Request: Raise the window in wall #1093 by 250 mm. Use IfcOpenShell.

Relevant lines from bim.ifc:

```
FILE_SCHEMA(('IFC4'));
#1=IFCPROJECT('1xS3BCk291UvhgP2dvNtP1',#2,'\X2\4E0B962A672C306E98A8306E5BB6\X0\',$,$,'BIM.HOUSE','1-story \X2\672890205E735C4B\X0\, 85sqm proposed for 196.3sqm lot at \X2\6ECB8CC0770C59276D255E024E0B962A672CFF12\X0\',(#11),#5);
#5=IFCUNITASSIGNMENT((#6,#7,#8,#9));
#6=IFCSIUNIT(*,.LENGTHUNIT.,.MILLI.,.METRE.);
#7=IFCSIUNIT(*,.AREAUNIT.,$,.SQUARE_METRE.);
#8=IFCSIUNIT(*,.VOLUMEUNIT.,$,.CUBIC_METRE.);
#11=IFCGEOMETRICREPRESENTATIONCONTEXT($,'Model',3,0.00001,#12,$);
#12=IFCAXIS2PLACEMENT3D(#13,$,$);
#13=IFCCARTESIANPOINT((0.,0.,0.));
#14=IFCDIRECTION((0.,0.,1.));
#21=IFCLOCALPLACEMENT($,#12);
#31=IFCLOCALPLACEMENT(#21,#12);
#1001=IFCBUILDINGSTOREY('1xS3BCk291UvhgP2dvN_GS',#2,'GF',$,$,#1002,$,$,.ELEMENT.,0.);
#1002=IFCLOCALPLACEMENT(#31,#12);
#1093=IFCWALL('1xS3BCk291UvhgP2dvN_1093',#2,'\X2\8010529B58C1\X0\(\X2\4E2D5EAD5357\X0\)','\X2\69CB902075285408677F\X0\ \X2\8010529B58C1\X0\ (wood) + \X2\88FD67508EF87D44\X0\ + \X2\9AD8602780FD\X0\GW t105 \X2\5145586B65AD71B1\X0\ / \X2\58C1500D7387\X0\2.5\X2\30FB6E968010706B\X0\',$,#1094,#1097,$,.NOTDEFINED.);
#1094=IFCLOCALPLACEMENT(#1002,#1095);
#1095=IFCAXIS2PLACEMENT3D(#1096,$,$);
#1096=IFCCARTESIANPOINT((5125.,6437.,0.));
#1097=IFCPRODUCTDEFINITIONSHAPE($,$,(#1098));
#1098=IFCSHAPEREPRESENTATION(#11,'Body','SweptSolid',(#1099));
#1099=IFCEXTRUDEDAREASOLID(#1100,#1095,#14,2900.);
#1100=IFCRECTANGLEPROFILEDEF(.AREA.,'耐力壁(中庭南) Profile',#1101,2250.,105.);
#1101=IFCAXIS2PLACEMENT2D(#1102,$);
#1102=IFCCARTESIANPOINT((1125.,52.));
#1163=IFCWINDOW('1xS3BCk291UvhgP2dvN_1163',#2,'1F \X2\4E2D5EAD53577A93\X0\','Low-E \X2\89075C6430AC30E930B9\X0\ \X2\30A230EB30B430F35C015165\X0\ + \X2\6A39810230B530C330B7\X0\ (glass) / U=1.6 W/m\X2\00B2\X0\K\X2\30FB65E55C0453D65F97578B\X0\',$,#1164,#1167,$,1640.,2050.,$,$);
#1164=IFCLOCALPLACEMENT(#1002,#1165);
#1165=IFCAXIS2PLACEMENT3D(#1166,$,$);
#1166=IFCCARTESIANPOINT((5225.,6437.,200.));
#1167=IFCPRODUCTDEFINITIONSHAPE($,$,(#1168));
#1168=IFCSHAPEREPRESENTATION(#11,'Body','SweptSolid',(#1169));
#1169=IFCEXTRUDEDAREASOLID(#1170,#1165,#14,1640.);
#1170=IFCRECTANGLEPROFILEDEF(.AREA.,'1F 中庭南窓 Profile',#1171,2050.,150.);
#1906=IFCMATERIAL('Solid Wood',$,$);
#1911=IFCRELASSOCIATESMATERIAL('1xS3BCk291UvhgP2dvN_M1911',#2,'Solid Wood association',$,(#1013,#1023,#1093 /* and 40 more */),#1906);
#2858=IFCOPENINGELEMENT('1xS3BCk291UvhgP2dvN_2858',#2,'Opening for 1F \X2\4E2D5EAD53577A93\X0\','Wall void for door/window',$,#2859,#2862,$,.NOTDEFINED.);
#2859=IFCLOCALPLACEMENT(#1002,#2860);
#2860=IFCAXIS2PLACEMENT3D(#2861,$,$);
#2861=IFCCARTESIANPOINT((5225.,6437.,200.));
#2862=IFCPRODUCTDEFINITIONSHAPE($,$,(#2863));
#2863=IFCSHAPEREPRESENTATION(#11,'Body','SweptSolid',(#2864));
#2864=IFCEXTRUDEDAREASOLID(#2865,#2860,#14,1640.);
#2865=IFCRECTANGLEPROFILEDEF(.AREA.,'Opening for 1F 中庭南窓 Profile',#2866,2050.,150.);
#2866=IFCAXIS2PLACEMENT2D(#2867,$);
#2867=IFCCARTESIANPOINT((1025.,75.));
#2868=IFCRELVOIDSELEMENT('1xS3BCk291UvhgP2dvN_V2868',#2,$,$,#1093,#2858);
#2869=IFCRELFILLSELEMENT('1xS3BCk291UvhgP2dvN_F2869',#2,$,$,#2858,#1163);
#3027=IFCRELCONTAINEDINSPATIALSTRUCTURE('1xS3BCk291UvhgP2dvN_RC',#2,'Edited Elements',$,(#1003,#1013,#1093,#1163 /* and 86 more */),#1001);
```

```python
import numpy as np
import ifcopenshell
import ifcopenshell.api.geometry
import ifcopenshell.util.placement
import ifcopenshell.util.unit

model = ifcopenshell.open("bim.ifc")
unit_scale = ifcopenshell.util.unit.calculate_unit_scale(model)

window = model.by_guid("1xS3BCk291UvhgP2dvN_1163")
opening = window.FillsVoids[0].RelatingOpeningElement
dz = 0.25 / unit_scale

shift = np.array([0.0, 0.0, dz])
# The window is not placed relative to its opening, so move both.
for product in (opening, window):
    matrix = ifcopenshell.util.placement.get_local_placement(product.ObjectPlacement)
    matrix[:3, 3] += shift
    ifcopenshell.api.geometry.edit_object_placement(model, product=product, matrix=matrix, is_si=False)

print(f"moved by {dz * unit_scale:+.3f} m")

model.write("bim_updated.ifc")
```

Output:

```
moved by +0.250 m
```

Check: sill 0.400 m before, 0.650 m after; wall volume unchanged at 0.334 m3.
